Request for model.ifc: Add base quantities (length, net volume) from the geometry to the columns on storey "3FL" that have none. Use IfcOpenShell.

First a look at what the model holds.

```python
import ifcopenshell
import ifcopenshell.util.element
import ifcopenshell.util.unit

model = ifcopenshell.open("model.ifc")
print(model.schema)
for unit_type in ("LENGTHUNIT", "AREAUNIT", "VOLUMEUNIT"):
    print(unit_type, ifcopenshell.util.unit.calculate_unit_scale(model, unit_type))
storey = next(s for s in model.by_type("IfcBuildingStorey") if s.Name == "3FL")
columns = [e for e in ifcopenshell.util.element.get_decomposition(storey) if e.is_a("IfcColumn")]
for e in sorted(columns, key=lambda e: e.id()):
    print(e.id(), e.is_a(), e.Name, list(ifcopenshell.util.element.get_psets(e, qtos_only=True)), sep=" | ")
```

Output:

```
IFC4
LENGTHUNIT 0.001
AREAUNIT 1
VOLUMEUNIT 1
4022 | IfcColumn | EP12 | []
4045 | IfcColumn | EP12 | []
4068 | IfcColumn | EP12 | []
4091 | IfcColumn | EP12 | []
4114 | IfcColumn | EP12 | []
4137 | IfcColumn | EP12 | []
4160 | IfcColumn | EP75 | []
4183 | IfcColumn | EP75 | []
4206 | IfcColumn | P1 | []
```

```python
import ifcopenshell
import ifcopenshell.api.pset
import ifcopenshell.geom
import ifcopenshell.util.element
import ifcopenshell.util.shape
import ifcopenshell.util.unit

model = ifcopenshell.open("model.ifc")
unit_scale = ifcopenshell.util.unit.calculate_unit_scale(model)
volume_scale = ifcopenshell.util.unit.calculate_unit_scale(model, "VOLUMEUNIT")
settings = ifcopenshell.geom.settings()

storey = next(s for s in model.by_type("IfcBuildingStorey") if s.Name == "3FL")
columns = [e for e in ifcopenshell.util.element.get_decomposition(storey) if e.is_a("IfcColumn")]

for e in sorted(columns, key=lambda e: e.id()):
    if ifcopenshell.util.element.get_psets(e, qtos_only=True, should_inherit=False):
        continue
    # Geometry comes back in metres, in the element's own axes.
    shape = ifcopenshell.geom.create_shape(settings, e)
    values = {
        "Length": ifcopenshell.util.shape.get_z(shape.geometry) / unit_scale,
        "NetVolume": ifcopenshell.util.shape.get_volume(shape.geometry) / volume_scale,
    }
    qto = ifcopenshell.api.pset.add_qto(model, product=e, name="Qto_ColumnBaseQuantities")
    ifcopenshell.api.pset.edit_qto(model, qto=qto, properties=values)
    print(e.id(), {k: round(v, 3) for k, v in values.items()})

model.write("model-out.ifc")
```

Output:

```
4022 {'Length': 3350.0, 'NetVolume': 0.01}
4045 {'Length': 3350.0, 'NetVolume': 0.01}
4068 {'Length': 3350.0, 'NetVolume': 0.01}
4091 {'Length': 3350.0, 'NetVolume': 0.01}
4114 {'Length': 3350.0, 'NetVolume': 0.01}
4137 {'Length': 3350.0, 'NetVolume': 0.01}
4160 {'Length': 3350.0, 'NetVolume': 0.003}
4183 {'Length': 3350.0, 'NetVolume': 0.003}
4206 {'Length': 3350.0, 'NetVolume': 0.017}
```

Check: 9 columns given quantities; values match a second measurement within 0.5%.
